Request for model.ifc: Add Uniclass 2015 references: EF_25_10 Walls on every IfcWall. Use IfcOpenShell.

First a look at what the model holds.

```python
import ifcopenshell

model = ifcopenshell.open("model.ifc")
print(model.schema)
print("classifications:", [c.Name for c in model.by_type("IfcClassification")])
for ifc_class in ("IfcDoor", "IfcRoof", "IfcStair", "IfcWall", "IfcWindow"):
    print(ifc_class, len(model.by_type(ifc_class)))
```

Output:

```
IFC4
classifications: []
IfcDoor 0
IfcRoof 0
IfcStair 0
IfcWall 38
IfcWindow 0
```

```python
import ifcopenshell
import ifcopenshell.api.classification

model = ifcopenshell.open("model.ifc")

system = ifcopenshell.api.classification.add_classification(model, classification="Uniclass 2015")

codes = {
    "IfcWall": ("EF_25_10", "Walls"),
}
for ifc_class, (code, name) in codes.items():
    products = model.by_type(ifc_class)
    ifcopenshell.api.classification.add_reference(
        model, products=products, classification=system, identification=code, name=name
    )
    print(code, len(products))

model.write("model_v2.ifc")
```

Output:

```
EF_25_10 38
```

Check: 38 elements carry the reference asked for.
